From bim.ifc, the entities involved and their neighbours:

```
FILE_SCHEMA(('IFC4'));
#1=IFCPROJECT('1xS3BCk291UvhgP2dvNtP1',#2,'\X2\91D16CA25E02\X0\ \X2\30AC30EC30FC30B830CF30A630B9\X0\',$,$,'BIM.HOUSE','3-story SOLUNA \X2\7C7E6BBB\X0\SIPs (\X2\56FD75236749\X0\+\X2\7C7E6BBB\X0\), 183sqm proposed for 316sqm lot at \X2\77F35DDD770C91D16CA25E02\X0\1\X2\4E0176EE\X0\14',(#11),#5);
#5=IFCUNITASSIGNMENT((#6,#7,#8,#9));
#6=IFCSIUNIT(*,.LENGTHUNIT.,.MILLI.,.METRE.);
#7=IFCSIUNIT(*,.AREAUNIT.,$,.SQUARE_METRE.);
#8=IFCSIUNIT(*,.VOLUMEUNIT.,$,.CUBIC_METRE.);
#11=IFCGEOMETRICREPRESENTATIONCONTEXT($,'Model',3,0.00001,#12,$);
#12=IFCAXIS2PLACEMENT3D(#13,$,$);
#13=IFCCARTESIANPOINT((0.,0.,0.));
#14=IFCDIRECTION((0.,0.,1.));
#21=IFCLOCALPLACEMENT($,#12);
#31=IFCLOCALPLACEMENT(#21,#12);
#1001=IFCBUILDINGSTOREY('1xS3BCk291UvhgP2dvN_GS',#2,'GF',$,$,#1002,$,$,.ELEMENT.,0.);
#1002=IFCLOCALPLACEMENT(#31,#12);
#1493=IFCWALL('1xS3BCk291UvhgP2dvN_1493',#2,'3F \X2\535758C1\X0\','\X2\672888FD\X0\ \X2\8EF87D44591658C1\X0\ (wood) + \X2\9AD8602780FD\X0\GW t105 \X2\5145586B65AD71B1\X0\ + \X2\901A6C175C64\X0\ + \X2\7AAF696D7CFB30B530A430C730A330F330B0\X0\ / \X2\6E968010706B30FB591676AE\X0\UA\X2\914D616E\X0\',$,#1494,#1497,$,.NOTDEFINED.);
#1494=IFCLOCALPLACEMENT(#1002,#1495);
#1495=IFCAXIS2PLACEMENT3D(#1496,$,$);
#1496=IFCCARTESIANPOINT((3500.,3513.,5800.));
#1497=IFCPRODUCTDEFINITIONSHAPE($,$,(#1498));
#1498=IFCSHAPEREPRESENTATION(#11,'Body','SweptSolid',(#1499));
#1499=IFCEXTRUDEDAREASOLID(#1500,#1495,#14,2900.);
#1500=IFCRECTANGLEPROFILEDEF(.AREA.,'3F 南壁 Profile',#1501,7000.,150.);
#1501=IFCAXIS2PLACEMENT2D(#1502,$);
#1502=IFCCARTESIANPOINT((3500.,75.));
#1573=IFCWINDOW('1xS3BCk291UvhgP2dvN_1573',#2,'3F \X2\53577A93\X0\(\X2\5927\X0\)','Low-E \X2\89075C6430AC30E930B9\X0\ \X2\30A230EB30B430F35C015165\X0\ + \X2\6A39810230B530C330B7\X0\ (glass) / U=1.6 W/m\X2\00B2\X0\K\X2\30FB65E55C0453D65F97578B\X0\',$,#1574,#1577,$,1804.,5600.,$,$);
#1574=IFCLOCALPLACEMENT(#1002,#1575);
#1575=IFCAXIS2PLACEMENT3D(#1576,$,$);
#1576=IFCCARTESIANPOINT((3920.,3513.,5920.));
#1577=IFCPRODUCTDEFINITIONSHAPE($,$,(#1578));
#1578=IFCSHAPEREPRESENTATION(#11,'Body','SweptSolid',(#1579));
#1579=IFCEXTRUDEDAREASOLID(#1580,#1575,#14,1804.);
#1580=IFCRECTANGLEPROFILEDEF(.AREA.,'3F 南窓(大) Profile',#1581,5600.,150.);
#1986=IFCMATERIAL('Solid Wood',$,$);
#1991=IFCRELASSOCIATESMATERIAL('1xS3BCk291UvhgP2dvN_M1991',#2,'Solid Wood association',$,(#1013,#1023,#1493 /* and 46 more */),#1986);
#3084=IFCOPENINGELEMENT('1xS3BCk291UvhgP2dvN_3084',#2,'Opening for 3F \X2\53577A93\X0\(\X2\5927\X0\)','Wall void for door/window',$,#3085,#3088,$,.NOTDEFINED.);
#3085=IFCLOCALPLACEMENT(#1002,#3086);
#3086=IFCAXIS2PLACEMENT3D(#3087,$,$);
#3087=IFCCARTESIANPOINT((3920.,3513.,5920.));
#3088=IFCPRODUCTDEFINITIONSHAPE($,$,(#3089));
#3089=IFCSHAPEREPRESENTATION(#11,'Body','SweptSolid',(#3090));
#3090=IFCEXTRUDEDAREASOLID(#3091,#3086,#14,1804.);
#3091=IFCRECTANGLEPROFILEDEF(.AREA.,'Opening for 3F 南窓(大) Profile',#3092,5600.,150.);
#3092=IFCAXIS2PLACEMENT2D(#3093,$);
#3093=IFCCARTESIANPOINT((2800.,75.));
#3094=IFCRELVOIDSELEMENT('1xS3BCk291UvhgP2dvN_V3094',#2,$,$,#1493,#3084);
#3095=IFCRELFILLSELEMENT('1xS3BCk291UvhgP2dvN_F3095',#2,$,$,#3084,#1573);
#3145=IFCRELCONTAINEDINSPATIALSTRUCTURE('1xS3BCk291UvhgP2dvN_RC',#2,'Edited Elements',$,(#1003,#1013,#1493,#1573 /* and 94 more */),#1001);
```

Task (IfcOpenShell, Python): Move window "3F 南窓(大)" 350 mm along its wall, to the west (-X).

```python
import ifcopenshell
import ifcopenshell.api.geometry
import ifcopenshell.util.placement
import ifcopenshell.util.unit

model = ifcopenshell.open("bim.ifc")
unit_scale = ifcopenshell.util.unit.calculate_unit_scale(model)

window = model.by_guid("1xS3BCk291UvhgP2dvN_1573")
opening = window.FillsVoids[0].RelatingOpeningElement
wall = opening.VoidsElements[0].RelatingBuildingElement

wall_matrix = ifcopenshell.util.placement.get_local_placement(wall.ObjectPlacement)
shift = wall_matrix[:3, 0] * -0.35 / unit_scale
before = ifcopenshell.util.placement.get_local_placement(window.ObjectPlacement)[:3, 3].copy()

# The window is not placed relative to its opening, so move both.
for product in (opening, window):
    matrix = ifcopenshell.util.placement.get_local_placement(product.ObjectPlacement)
    matrix[:3, 3] += shift
    ifcopenshell.api.geometry.edit_object_placement(model, product=product, matrix=matrix, is_si=False)

after = ifcopenshell.util.placement.get_local_placement(window.ObjectPlacement)[:3, 3]
print("window moved by", (after - before).round(3) + 0.0)

model.write("bim_rev.ifc")
```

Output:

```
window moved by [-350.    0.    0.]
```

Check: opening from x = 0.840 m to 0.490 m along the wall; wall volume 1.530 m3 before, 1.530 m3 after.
